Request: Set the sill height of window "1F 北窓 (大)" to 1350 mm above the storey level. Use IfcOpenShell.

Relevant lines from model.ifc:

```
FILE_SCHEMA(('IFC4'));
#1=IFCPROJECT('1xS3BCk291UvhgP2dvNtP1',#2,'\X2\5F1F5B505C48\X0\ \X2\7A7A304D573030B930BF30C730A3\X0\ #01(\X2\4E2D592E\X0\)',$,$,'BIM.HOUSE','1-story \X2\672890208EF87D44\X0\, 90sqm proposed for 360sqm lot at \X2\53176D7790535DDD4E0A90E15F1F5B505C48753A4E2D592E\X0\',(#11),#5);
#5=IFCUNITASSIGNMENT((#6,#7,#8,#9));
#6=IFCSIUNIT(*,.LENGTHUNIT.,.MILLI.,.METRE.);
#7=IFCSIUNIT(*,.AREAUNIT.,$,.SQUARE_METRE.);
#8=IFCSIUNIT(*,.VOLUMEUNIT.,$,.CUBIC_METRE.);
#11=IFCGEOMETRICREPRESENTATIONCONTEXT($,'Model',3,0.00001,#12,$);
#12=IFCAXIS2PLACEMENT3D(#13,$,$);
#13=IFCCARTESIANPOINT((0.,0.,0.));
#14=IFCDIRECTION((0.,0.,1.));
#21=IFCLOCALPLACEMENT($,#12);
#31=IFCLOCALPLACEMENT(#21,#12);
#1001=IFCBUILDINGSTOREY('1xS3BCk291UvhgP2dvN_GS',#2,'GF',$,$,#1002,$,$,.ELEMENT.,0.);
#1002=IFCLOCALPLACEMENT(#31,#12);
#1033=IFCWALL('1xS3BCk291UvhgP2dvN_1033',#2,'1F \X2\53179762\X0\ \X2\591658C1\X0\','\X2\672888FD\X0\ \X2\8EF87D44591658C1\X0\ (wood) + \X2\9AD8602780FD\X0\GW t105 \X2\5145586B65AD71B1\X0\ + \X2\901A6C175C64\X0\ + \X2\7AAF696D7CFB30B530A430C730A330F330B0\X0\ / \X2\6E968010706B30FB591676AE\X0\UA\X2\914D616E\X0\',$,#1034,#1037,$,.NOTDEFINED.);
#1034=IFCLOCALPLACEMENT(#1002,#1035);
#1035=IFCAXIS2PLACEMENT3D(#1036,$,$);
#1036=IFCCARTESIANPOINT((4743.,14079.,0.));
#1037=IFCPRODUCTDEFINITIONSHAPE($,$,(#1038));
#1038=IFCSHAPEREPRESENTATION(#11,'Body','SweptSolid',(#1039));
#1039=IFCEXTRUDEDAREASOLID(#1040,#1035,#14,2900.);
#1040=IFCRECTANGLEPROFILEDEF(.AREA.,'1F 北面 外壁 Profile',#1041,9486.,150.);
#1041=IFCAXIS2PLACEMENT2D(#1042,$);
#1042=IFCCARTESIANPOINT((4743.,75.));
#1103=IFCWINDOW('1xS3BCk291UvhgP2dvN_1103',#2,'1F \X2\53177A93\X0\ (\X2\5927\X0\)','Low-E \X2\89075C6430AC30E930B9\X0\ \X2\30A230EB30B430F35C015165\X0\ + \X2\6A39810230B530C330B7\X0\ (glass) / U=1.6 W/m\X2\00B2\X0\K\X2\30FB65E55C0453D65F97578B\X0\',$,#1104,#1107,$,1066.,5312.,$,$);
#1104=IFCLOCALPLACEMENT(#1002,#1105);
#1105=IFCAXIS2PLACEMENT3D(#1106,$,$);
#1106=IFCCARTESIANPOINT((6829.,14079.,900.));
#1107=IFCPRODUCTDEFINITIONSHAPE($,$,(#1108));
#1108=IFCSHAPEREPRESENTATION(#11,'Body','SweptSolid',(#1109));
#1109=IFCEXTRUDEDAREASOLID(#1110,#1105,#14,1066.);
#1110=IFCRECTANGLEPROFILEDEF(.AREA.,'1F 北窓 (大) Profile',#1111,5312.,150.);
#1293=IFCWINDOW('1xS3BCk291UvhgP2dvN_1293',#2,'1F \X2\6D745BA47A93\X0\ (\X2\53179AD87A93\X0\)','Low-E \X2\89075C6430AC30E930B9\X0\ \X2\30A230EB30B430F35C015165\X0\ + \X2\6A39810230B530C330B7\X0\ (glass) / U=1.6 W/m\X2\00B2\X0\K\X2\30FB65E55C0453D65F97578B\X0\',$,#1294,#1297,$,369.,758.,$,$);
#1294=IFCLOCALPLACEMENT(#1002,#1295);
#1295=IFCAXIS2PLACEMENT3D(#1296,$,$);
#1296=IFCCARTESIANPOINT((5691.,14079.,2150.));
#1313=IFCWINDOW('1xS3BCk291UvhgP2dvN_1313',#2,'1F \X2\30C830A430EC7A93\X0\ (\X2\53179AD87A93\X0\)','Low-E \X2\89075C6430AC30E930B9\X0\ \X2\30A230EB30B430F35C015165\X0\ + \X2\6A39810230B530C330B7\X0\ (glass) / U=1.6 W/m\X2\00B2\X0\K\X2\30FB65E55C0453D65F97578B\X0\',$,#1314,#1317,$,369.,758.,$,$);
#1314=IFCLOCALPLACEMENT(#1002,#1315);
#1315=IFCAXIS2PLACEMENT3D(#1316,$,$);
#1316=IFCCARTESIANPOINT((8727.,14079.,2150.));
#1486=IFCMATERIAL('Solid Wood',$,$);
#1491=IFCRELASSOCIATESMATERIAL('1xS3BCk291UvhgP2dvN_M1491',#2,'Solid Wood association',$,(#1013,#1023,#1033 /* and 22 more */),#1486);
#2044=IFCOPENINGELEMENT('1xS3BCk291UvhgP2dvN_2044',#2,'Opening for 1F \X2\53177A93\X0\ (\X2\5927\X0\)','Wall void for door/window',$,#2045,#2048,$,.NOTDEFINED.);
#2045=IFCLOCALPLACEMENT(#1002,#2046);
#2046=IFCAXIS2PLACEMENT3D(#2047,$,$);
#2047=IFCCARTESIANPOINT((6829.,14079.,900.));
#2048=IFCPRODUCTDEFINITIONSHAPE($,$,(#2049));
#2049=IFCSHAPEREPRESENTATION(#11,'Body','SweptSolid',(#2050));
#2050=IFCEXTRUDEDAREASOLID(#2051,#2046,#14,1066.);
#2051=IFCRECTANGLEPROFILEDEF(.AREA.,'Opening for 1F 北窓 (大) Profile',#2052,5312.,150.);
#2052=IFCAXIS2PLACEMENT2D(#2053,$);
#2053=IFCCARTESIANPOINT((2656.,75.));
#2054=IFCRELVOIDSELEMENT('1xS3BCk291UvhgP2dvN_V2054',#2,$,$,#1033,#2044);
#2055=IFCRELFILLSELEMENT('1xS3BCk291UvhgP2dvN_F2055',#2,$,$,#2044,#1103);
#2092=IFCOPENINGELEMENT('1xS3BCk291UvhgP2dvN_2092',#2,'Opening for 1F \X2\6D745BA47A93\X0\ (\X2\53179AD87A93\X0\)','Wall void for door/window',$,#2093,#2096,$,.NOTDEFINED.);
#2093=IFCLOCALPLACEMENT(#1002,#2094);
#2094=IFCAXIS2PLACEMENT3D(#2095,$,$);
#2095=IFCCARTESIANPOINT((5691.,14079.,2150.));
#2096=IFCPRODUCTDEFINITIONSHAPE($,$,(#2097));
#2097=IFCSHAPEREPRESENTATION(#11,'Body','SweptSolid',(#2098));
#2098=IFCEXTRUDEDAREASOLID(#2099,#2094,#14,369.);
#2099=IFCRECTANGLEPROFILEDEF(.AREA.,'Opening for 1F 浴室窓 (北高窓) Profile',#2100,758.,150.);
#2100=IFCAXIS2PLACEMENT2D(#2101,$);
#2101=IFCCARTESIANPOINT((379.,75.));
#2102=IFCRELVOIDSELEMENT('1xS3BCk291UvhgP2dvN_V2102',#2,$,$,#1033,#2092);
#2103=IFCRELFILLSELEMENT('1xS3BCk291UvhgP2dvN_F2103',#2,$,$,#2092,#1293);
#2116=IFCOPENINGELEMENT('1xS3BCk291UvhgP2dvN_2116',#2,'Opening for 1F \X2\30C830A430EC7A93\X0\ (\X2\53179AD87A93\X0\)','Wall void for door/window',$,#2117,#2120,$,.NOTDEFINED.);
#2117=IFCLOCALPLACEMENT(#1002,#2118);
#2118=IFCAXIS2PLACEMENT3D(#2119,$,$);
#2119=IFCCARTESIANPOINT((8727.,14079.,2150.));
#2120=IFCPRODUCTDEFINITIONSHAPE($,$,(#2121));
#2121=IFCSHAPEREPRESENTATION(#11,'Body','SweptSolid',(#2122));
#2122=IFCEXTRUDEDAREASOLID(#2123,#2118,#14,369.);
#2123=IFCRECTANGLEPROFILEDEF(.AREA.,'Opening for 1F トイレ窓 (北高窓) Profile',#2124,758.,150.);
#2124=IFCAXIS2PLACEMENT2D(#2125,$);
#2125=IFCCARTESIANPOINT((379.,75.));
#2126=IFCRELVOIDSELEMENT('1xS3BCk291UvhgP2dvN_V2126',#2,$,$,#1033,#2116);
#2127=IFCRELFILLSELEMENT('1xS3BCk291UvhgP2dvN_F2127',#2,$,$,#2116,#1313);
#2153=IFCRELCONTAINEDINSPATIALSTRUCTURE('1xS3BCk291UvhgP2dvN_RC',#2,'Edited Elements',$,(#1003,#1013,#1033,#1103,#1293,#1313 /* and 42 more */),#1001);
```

```python
import numpy as np
import ifcopenshell
import ifcopenshell.api.geometry
import ifcopenshell.geom
import ifcopenshell.util.element
import ifcopenshell.util.placement
import ifcopenshell.util.shape
import ifcopenshell.util.unit

model = ifcopenshell.open("model.ifc")
unit_scale = ifcopenshell.util.unit.calculate_unit_scale(model)

window = model.by_id(1103)
opening = window.FillsVoids[0].RelatingOpeningElement
storey = ifcopenshell.util.element.get_container(window, ifc_class="IfcBuildingStorey")
level = ifcopenshell.util.placement.get_local_placement(storey.ObjectPlacement)[2, 3]

# The opening's origin need not be at the sill, so measure its lowest point.
shape = ifcopenshell.geom.create_shape(ifcopenshell.geom.settings(), opening)
bottom = ifcopenshell.util.shape.get_shape_bottom_elevation(shape, shape.geometry) / unit_scale
dz = level + 1350.0 - bottom

shift = np.array([0.0, 0.0, dz])
# The window is not placed relative to its opening, so move both.
for product in (opening, window):
    matrix = ifcopenshell.util.placement.get_local_placement(product.ObjectPlacement)
    matrix[:3, 3] += shift
    ifcopenshell.api.geometry.edit_object_placement(model, product=product, matrix=matrix, is_si=False)

print(f"moved by {dz * unit_scale:+.3f} m")

model.write("model_rev.ifc")
```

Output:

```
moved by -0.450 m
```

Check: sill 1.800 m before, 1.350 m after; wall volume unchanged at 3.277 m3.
